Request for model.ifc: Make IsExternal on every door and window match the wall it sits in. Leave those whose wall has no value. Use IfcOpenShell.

First a look at what the model holds.

```python
import ifcopenshell
import ifcopenshell.util.element

model = ifcopenshell.open("model.ifc")
print(model.schema)
seen = {}
for e in model.by_type("IfcDoor") + model.by_type("IfcWindow"):
    if not e.FillsVoids:
        continue
    host = e.FillsVoids[0].RelatingOpeningElement.VoidsElements[0].RelatingBuildingElement
    own = ifcopenshell.util.element.get_pset(e, f"Pset_{e.is_a()[3:].removesuffix('StandardCase')}Common", "IsExternal")
    wall = ifcopenshell.util.element.get_pset(host, "Pset_WallCommon", "IsExternal")
    seen[e.is_a(), own, wall] = seen.get((e.is_a(), own, wall), 0) + 1
for (cls, own, wall), count in sorted(seen.items(), key=str):
    print(count, cls, "IsExternal:", own, "| host wall:", wall)
```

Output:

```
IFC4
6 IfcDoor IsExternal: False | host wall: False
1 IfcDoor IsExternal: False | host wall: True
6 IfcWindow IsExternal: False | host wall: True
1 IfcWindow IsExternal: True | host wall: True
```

```python
import ifcopenshell
import ifcopenshell.api.pset
import ifcopenshell.util.element

model = ifcopenshell.open("model.ifc")

count = 0
for ifc_class, pset_name in (("IfcDoor", "Pset_DoorCommon"), ("IfcWindow", "Pset_WindowCommon")):
    for e in model.by_type(ifc_class):
        if not e.FillsVoids:
            continue
        host = e.FillsVoids[0].RelatingOpeningElement.VoidsElements[0].RelatingBuildingElement
        external = ifcopenshell.util.element.get_pset(host, "Pset_WallCommon", "IsExternal")
        if external is None or ifcopenshell.util.element.get_pset(e, pset_name, "IsExternal") == external:
            continue
        pset = ifcopenshell.api.pset.add_pset(model, product=e, name=pset_name)
        ifcopenshell.api.pset.edit_pset(model, pset=pset, properties={"IsExternal": external})
        count += 1

print(count, "updated")

model.write("model_v2.ifc")
```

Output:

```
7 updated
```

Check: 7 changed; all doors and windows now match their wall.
